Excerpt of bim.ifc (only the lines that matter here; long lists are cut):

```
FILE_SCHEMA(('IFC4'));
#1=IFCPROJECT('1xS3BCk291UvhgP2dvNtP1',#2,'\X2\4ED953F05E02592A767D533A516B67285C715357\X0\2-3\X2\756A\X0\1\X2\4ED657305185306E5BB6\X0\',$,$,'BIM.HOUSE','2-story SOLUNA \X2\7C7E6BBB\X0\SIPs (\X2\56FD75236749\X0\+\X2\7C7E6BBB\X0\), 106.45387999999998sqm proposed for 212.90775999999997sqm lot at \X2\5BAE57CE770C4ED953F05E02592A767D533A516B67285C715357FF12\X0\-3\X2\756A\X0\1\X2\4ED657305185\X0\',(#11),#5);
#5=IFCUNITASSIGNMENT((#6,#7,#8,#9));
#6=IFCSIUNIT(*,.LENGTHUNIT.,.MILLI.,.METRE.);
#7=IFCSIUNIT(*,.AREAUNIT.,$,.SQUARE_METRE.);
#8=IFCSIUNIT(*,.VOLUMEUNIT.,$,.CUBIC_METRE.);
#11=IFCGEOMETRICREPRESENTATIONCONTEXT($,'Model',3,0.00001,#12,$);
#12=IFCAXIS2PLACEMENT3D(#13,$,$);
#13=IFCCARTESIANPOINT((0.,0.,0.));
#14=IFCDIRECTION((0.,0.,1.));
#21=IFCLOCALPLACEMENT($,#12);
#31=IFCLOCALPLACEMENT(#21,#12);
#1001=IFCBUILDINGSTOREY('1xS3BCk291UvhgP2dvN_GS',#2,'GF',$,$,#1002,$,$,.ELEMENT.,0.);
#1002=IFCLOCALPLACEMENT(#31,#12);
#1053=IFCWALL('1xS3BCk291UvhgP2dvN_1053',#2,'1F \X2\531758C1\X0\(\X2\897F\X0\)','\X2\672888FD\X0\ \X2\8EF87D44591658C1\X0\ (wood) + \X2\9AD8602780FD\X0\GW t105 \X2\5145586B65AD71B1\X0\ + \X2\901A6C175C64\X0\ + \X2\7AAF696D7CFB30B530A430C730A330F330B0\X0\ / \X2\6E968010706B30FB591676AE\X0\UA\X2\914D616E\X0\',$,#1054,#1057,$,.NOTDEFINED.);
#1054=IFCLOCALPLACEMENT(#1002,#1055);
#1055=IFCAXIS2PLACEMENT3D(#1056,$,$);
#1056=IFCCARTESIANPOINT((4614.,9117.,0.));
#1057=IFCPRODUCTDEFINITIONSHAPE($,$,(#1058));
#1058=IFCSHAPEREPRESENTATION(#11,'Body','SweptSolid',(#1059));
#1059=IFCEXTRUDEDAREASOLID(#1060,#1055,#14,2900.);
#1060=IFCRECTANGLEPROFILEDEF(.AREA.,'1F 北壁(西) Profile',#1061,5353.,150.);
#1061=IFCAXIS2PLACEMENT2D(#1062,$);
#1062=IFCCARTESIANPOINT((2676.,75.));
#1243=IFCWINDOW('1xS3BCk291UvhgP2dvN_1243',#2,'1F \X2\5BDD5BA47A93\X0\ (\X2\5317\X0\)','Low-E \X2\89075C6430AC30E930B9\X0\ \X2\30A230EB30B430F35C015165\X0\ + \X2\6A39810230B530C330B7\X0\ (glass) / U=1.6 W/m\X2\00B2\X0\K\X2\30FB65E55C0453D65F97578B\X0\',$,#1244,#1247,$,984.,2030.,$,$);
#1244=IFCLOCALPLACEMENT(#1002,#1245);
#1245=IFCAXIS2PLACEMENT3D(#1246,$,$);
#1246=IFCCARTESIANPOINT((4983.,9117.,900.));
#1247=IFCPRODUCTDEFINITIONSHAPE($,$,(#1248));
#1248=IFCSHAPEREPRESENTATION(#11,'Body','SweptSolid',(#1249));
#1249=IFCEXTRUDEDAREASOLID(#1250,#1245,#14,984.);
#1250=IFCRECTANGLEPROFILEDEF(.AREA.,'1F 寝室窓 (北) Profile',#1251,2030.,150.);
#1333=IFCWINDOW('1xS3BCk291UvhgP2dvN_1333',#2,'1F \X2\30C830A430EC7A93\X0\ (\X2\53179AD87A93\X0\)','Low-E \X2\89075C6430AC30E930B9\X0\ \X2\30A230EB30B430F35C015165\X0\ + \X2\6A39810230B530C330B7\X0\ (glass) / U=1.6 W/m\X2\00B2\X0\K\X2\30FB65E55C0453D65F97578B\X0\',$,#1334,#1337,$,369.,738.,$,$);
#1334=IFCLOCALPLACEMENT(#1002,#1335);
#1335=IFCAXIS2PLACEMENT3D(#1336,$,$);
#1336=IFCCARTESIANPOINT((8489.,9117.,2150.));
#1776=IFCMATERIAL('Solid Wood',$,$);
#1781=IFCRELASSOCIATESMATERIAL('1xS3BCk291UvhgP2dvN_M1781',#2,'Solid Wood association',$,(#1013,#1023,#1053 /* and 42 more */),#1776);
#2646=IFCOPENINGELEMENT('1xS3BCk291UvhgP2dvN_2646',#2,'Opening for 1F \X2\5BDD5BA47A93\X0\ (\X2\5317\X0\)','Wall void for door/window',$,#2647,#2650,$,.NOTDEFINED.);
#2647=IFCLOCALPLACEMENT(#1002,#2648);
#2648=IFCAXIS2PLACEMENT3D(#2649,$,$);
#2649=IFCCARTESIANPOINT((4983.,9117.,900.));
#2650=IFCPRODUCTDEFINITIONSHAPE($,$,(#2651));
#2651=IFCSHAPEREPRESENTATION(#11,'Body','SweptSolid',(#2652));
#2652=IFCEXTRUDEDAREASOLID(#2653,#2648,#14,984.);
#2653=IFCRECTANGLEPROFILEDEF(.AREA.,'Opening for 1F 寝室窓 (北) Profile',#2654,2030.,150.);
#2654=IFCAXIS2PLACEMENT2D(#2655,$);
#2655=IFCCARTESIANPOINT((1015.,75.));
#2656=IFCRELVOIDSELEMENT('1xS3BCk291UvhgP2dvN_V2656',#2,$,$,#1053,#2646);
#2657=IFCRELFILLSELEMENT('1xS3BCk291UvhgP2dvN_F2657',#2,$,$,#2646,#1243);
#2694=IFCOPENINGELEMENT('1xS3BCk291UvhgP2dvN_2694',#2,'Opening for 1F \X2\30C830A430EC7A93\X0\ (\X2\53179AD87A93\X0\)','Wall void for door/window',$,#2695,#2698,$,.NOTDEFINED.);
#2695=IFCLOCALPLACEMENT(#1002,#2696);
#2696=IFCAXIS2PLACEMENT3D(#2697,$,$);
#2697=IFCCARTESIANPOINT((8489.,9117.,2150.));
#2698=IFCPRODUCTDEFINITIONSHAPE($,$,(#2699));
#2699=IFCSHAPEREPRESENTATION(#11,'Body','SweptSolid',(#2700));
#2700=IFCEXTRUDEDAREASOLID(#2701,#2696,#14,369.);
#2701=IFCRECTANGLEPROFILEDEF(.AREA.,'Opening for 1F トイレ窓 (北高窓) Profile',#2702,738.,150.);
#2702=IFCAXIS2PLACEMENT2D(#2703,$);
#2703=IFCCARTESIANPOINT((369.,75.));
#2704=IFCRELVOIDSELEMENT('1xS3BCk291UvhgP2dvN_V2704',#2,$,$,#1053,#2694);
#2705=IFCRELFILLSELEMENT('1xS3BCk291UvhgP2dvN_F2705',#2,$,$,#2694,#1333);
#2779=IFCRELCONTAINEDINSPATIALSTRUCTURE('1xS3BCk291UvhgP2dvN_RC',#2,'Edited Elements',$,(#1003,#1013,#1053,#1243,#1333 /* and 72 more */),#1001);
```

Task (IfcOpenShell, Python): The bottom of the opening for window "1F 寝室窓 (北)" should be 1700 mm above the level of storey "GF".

```python
import numpy as np
import ifcopenshell
import ifcopenshell.api.geometry
import ifcopenshell.geom
import ifcopenshell.util.element
import ifcopenshell.util.placement
import ifcopenshell.util.shape
import ifcopenshell.util.unit

model = ifcopenshell.open("bim.ifc")
unit_scale = ifcopenshell.util.unit.calculate_unit_scale(model)

window = model.by_id(1243)
opening = window.FillsVoids[0].RelatingOpeningElement
storey = ifcopenshell.util.element.get_container(window, ifc_class="IfcBuildingStorey")
level = ifcopenshell.util.placement.get_local_placement(storey.ObjectPlacement)[2, 3]

# The opening's origin need not be at the sill, so measure its lowest point.
shape = ifcopenshell.geom.create_shape(ifcopenshell.geom.settings(), opening)
bottom = ifcopenshell.util.shape.get_shape_bottom_elevation(shape, shape.geometry) / unit_scale
dz = level + 1.7 / unit_scale - bottom

shift = np.array([0.0, 0.0, dz])
# The window is not placed relative to its opening, so move both.
for product in (opening, window):
    matrix = ifcopenshell.util.placement.get_local_placement(product.ObjectPlacement)
    matrix[:3, 3] += shift
    ifcopenshell.api.geometry.edit_object_placement(model, product=product, matrix=matrix, is_si=False)

print(f"moved by {dz * unit_scale:+.3f} m")

model.write("bim_edited.ifc")
```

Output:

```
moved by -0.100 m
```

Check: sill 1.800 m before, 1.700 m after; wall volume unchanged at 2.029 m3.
